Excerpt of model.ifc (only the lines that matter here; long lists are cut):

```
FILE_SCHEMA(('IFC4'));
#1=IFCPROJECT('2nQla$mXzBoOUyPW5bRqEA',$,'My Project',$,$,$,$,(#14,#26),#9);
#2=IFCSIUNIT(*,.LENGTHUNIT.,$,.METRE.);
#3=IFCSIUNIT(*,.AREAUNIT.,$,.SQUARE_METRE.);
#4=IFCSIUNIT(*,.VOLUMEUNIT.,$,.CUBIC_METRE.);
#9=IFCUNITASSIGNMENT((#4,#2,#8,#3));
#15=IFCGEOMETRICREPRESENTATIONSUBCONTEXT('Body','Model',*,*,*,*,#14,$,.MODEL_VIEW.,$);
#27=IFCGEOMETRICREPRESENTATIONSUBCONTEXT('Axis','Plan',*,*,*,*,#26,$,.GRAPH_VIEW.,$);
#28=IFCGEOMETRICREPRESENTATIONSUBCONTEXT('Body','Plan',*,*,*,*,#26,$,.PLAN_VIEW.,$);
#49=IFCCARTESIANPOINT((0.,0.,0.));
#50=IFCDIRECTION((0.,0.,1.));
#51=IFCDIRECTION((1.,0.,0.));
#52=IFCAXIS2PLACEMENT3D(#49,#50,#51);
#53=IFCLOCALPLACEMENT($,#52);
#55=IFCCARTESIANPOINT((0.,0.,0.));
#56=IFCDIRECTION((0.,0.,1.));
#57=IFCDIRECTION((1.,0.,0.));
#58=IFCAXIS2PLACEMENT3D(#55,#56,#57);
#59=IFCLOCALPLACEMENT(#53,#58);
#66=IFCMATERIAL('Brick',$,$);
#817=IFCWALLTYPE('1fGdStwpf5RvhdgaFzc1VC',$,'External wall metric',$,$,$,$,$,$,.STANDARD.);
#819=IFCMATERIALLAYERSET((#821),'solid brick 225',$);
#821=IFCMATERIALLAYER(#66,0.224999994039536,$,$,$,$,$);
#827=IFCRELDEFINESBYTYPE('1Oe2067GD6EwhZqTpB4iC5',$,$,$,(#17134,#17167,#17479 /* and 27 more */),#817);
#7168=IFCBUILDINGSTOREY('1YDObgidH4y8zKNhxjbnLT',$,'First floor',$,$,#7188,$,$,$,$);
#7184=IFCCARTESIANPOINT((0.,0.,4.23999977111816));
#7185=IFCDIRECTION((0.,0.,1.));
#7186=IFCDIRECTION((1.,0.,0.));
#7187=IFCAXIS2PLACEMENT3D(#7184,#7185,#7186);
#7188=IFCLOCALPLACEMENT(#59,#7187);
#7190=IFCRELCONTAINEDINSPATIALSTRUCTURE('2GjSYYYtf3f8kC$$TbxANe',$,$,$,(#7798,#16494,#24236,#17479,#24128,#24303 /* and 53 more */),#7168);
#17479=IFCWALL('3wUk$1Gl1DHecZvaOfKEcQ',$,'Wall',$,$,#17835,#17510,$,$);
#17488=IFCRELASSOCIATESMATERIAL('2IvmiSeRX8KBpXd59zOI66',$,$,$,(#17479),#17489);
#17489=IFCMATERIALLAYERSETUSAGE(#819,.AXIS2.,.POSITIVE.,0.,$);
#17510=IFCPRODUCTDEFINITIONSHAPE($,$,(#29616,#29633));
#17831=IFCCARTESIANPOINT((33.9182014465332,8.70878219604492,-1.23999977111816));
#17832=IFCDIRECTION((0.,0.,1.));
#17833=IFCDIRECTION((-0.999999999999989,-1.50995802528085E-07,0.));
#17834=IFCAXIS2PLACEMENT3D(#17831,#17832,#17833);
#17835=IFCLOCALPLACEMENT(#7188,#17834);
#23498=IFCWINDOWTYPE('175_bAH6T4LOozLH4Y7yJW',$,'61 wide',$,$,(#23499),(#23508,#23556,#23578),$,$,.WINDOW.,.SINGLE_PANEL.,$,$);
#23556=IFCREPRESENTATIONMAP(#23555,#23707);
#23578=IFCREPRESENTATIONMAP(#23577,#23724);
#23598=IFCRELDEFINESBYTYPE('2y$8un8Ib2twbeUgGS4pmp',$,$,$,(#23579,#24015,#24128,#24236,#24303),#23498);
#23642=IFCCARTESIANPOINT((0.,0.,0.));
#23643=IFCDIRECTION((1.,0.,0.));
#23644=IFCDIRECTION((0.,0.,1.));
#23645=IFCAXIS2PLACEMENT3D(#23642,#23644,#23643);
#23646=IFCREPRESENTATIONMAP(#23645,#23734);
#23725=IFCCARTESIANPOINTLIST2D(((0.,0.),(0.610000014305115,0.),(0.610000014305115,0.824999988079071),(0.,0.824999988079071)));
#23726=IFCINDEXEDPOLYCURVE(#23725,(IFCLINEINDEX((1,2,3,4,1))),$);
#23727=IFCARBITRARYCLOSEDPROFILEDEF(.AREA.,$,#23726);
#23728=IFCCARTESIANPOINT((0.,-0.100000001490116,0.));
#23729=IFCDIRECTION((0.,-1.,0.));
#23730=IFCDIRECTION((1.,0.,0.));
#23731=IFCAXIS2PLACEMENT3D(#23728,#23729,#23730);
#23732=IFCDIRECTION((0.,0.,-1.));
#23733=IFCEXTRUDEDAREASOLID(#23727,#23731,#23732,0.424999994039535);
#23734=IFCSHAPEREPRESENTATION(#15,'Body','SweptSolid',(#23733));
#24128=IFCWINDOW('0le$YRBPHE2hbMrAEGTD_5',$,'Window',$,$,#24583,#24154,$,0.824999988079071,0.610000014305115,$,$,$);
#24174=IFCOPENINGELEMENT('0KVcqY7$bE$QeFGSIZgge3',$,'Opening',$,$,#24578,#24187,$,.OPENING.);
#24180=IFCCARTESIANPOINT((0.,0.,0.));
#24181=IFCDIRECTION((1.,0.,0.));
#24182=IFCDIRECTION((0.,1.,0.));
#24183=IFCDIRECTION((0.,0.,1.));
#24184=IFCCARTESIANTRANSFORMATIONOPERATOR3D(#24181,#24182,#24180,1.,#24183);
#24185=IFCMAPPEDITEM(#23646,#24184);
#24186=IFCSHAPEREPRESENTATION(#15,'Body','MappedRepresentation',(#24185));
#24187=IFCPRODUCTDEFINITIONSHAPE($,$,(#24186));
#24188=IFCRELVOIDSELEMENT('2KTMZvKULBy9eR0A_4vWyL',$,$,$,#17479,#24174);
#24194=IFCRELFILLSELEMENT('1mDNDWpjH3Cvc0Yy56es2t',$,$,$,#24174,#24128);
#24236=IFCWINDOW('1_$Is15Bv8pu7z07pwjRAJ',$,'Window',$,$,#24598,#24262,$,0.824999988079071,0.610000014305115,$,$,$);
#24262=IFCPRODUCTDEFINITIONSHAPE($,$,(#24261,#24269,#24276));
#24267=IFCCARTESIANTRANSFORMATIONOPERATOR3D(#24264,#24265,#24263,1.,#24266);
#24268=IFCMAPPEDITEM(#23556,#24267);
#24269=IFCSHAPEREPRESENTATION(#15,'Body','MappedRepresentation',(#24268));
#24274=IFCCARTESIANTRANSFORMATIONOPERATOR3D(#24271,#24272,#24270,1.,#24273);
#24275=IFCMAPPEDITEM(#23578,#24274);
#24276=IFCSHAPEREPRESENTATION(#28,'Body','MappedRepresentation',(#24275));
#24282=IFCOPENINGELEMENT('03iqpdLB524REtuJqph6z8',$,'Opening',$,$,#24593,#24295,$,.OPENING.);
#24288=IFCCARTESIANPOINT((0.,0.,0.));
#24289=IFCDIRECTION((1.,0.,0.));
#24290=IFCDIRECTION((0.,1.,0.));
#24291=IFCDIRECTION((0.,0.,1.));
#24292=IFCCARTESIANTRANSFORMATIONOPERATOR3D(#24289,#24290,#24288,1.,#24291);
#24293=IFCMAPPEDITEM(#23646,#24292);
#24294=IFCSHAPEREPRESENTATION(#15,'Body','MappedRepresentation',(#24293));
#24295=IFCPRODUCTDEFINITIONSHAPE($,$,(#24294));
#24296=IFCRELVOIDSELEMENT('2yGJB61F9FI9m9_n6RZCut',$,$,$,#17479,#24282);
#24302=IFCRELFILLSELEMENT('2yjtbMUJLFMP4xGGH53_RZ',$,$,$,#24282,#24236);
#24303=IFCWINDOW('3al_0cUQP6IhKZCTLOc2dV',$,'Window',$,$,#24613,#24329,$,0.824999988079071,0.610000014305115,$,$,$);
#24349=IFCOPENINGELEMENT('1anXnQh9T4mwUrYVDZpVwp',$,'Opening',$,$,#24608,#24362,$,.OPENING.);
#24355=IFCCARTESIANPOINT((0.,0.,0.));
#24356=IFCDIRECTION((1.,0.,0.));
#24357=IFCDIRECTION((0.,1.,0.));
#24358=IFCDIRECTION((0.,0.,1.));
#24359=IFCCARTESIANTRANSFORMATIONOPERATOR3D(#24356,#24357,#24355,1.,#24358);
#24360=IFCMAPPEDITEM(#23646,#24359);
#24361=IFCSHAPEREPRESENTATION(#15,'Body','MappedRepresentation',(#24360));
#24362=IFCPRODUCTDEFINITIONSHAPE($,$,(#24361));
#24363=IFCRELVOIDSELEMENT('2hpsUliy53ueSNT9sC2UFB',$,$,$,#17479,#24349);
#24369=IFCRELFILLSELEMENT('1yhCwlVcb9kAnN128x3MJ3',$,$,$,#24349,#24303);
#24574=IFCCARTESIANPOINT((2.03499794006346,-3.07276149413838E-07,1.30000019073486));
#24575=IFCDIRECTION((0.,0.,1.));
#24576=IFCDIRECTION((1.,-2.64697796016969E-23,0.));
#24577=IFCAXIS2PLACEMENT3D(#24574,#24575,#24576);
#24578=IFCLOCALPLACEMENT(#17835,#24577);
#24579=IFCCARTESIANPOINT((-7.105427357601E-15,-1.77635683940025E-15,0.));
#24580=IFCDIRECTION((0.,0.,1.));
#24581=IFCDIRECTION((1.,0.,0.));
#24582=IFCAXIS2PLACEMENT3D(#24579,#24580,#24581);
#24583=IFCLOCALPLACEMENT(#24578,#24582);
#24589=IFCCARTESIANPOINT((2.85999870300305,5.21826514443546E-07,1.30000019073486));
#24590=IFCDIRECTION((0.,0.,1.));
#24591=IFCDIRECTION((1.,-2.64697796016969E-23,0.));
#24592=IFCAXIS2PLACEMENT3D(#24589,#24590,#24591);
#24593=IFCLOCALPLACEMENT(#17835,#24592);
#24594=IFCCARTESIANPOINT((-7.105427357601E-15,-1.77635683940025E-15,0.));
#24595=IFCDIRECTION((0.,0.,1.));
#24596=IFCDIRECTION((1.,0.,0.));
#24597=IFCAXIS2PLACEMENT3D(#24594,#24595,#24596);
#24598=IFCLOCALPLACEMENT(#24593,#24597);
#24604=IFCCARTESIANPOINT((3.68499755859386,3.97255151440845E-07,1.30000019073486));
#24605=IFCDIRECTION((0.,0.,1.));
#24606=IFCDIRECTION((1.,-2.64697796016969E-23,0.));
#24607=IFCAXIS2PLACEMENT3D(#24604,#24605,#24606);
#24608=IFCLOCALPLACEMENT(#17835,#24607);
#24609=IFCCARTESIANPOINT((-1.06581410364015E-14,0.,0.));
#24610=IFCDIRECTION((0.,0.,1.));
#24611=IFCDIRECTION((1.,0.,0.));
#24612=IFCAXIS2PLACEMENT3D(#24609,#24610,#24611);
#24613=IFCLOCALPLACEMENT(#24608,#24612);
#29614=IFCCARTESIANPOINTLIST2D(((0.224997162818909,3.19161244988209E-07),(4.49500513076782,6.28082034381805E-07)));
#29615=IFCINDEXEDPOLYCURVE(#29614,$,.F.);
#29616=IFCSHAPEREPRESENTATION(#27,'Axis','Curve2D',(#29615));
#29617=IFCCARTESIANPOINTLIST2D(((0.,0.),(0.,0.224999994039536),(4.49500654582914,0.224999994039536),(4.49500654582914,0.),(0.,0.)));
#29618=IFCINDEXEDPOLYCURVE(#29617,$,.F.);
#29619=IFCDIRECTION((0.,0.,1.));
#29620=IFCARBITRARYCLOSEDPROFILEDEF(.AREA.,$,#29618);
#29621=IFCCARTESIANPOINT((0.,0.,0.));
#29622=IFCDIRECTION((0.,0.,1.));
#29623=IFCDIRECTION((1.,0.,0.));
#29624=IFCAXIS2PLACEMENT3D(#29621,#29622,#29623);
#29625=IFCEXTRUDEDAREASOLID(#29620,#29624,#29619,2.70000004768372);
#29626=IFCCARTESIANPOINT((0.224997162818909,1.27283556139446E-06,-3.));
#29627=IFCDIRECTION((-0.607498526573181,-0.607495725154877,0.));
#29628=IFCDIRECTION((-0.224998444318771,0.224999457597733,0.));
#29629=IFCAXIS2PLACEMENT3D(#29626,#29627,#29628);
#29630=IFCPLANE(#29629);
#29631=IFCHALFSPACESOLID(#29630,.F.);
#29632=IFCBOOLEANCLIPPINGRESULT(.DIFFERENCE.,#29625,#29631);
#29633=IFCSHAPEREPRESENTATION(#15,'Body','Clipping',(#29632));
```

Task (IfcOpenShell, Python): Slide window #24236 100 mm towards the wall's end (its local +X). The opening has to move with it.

```python
import ifcopenshell
import ifcopenshell.api.geometry
import ifcopenshell.util.placement
import ifcopenshell.util.unit

model = ifcopenshell.open("model.ifc")
unit_scale = ifcopenshell.util.unit.calculate_unit_scale(model)

window = model.by_id(24236)
opening = window.FillsVoids[0].RelatingOpeningElement
wall = opening.VoidsElements[0].RelatingBuildingElement

wall_matrix = ifcopenshell.util.placement.get_local_placement(wall.ObjectPlacement)
shift = wall_matrix[:3, 0] * 0.1 / unit_scale
before = ifcopenshell.util.placement.get_local_placement(window.ObjectPlacement)[:3, 3].copy()

# The window is placed relative to its opening, so it follows when the opening moves.
matrix = ifcopenshell.util.placement.get_local_placement(opening.ObjectPlacement)
matrix[:3, 3] += shift
ifcopenshell.api.geometry.edit_object_placement(
    model, product=opening, matrix=matrix, is_si=False, should_transform_children=True
)

after = ifcopenshell.util.placement.get_local_placement(window.ObjectPlacement)[:3, 3]
print("window moved by", (after - before).round(3) + 0.0)

model.write("model_v2.ifc")
```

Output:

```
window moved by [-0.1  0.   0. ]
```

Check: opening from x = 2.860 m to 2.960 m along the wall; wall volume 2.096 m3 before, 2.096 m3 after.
